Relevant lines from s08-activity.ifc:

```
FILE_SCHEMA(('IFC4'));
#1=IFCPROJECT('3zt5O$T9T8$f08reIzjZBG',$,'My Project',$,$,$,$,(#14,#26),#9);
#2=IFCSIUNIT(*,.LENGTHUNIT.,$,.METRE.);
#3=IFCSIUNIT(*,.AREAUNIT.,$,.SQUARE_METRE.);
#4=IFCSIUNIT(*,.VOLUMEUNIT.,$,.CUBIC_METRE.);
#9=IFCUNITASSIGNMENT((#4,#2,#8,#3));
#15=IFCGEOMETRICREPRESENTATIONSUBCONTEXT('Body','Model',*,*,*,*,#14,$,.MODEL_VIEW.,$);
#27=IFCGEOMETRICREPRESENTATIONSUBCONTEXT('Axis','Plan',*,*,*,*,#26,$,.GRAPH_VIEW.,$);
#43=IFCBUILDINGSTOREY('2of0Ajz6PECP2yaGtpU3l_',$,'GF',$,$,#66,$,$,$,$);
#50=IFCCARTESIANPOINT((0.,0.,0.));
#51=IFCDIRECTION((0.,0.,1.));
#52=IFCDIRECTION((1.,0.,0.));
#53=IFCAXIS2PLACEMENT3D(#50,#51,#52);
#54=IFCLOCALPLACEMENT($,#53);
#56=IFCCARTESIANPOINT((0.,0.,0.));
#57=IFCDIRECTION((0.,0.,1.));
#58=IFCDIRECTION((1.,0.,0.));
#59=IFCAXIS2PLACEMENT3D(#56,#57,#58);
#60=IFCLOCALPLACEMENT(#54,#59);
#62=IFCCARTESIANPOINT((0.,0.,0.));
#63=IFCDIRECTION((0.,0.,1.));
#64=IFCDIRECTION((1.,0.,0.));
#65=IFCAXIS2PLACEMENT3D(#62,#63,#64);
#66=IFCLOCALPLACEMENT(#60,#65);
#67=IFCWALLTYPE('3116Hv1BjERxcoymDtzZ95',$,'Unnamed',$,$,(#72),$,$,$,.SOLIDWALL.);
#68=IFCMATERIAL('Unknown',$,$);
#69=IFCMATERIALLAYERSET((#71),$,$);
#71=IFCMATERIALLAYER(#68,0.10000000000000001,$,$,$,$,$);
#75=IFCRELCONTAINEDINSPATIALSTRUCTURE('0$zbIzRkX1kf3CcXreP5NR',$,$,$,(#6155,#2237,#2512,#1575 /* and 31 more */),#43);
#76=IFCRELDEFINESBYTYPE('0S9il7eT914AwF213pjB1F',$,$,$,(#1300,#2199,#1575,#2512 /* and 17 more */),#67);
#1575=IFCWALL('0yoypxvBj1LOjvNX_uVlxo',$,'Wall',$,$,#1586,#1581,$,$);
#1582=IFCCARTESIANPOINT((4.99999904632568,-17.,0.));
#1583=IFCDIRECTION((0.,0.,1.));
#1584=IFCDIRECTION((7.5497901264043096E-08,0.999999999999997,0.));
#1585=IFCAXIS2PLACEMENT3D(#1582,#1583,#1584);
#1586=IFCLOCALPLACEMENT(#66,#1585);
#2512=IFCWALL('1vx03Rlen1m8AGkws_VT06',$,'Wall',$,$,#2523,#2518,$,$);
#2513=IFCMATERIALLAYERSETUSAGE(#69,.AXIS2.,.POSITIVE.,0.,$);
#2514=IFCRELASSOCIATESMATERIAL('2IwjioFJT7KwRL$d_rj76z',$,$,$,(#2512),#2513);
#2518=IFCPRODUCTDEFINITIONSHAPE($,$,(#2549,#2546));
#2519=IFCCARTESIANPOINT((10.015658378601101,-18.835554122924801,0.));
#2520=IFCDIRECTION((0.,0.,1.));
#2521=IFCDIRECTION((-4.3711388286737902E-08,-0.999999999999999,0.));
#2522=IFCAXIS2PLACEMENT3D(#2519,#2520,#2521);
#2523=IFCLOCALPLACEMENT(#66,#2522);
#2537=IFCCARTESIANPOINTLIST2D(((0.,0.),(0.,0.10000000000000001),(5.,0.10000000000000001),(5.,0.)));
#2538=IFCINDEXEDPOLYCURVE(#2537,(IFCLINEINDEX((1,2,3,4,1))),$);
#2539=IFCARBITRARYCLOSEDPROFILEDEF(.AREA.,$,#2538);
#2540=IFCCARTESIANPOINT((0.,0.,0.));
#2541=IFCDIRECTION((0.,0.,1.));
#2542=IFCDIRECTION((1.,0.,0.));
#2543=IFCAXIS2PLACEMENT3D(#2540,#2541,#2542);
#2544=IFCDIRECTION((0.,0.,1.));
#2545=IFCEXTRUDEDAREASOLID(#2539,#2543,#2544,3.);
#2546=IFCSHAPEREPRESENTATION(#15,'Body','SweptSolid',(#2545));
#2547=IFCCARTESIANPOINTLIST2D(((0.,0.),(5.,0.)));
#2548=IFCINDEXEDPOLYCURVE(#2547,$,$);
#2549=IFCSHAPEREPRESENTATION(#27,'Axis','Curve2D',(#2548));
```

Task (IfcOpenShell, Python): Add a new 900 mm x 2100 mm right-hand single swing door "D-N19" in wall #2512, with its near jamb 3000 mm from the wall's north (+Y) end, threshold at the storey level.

```python
import numpy as np
import ifcopenshell
import ifcopenshell.api.feature
import ifcopenshell.api.geometry
import ifcopenshell.api.root
import ifcopenshell.api.spatial
import ifcopenshell.geom
import ifcopenshell.util.element
import ifcopenshell.util.placement
import ifcopenshell.util.representation
import ifcopenshell.util.shape
import ifcopenshell.util.unit

model = ifcopenshell.open("s08-activity.ifc")
unit_scale = ifcopenshell.util.unit.calculate_unit_scale(model)
settings = ifcopenshell.geom.settings()


def volume(element):
    """Net volume in cubic metres, openings subtracted."""
    shape = ifcopenshell.geom.create_shape(settings, element)
    return ifcopenshell.util.shape.get_volume(shape.geometry)


wall = model.by_guid("1vx03Rlen1m8AGkws_VT06")
storey = ifcopenshell.util.element.get_container(wall, ifc_class="IfcBuildingStorey")
context = ifcopenshell.util.representation.get_context(model, "Model", "Body", "MODEL_VIEW")
before = volume(wall)

width, height, from_end, sill = 0.9, 2.1, 3, 0.0  # metres

# The wall runs along its own X axis, and the end named is its -X end.
wall_shape = ifcopenshell.geom.create_shape(settings, wall)
x, y, z = ifcopenshell.util.shape.get_vertices(wall_shape.geometry).T
start = x.min() + from_end
face, thickness = float(y.min()), float(y.max() - y.min())
wall_matrix = ifcopenshell.util.placement.get_local_placement(wall.ObjectPlacement)
level = ifcopenshell.util.placement.get_local_placement(storey.ObjectPlacement)[2, 3]


def in_wall(x, y):
    """Placement at x, y metres in the wall's axes, at sill height."""
    matrix = wall_matrix.copy()
    matrix[:, 3] = wall_matrix @ np.array([x / unit_scale, y / unit_scale, 0.0, 1.0])
    matrix[2, 3] = level + sill / unit_scale
    return matrix


# Opening: a box that overshoots both wall faces by 50 mm.
opening = ifcopenshell.api.root.create_entity(model, ifc_class="IfcOpeningElement", predefined_type="OPENING")
box = ifcopenshell.api.geometry.add_wall_representation(
    model, context=context, length=width, height=height, thickness=thickness + 0.1
)
ifcopenshell.api.geometry.assign_representation(model, product=opening, representation=box)
ifcopenshell.api.geometry.edit_object_placement(model, product=opening, matrix=in_wall(start, face - 0.05), is_si=False)
ifcopenshell.api.feature.add_feature(model, feature=opening, element=wall)

door = ifcopenshell.api.root.create_entity(model, ifc_class="IfcDoor", name="D-N19", predefined_type="DOOR")
door.OverallWidth, door.OverallHeight = width / unit_scale, height / unit_scale
door.OperationType = "SINGLE_SWING_RIGHT"
body = ifcopenshell.api.geometry.add_door_representation(
    model,
    context=context,
    overall_width=door.OverallWidth,
    overall_height=door.OverallHeight,
    operation_type="SINGLE_SWING_RIGHT",
    lining_properties={"LiningDepth": thickness / unit_scale, "ThresholdDepth": thickness / unit_scale},
)
ifcopenshell.api.geometry.assign_representation(model, product=door, representation=body)
ifcopenshell.api.spatial.assign_container(model, products=[door], relating_structure=storey)
ifcopenshell.api.feature.add_filling(model, opening=opening, element=door)

# The lining spans the wall, so the door starts at the wall face.
ifcopenshell.api.geometry.edit_object_placement(model, product=door, matrix=in_wall(start, face), is_si=False)

after = volume(wall)

print(f"wall volume {before:.3f} -> {after:.3f} m3")

model.write("s08-activity_v2.ifc")
```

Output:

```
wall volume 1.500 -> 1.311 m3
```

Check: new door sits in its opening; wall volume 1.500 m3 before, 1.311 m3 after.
